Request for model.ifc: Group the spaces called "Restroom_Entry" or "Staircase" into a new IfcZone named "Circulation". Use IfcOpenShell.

First a look at what the model holds.

```python
import ifcopenshell

model = ifcopenshell.open("model.ifc")
print(model.schema)
seen = {}
for space in model.by_type("IfcSpace"):
    seen[space.LongName] = seen.get(space.LongName, 0) + 1
for name, count in sorted(seen.items(), key=str):
    print(count, "x", name)
print("zones:", [z.Name for z in model.by_type("IfcZone")][:20])
```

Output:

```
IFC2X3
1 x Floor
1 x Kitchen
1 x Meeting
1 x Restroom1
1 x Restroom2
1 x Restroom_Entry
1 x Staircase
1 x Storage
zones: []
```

```python
import ifcopenshell
import ifcopenshell.api.group
import ifcopenshell.api.root

model = ifcopenshell.open("model.ifc")

names = {"Restroom_Entry", "Staircase"}
spaces = [s for s in model.by_type("IfcSpace") if s.LongName in names]

zone = ifcopenshell.api.root.create_entity(model, ifc_class="IfcZone", name="Circulation")
ifcopenshell.api.group.assign_group(model, products=spaces, group=zone)
print(len(spaces), "spaces in", zone.Name)

model.write("model_v2.ifc")
```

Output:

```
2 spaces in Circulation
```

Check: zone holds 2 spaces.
